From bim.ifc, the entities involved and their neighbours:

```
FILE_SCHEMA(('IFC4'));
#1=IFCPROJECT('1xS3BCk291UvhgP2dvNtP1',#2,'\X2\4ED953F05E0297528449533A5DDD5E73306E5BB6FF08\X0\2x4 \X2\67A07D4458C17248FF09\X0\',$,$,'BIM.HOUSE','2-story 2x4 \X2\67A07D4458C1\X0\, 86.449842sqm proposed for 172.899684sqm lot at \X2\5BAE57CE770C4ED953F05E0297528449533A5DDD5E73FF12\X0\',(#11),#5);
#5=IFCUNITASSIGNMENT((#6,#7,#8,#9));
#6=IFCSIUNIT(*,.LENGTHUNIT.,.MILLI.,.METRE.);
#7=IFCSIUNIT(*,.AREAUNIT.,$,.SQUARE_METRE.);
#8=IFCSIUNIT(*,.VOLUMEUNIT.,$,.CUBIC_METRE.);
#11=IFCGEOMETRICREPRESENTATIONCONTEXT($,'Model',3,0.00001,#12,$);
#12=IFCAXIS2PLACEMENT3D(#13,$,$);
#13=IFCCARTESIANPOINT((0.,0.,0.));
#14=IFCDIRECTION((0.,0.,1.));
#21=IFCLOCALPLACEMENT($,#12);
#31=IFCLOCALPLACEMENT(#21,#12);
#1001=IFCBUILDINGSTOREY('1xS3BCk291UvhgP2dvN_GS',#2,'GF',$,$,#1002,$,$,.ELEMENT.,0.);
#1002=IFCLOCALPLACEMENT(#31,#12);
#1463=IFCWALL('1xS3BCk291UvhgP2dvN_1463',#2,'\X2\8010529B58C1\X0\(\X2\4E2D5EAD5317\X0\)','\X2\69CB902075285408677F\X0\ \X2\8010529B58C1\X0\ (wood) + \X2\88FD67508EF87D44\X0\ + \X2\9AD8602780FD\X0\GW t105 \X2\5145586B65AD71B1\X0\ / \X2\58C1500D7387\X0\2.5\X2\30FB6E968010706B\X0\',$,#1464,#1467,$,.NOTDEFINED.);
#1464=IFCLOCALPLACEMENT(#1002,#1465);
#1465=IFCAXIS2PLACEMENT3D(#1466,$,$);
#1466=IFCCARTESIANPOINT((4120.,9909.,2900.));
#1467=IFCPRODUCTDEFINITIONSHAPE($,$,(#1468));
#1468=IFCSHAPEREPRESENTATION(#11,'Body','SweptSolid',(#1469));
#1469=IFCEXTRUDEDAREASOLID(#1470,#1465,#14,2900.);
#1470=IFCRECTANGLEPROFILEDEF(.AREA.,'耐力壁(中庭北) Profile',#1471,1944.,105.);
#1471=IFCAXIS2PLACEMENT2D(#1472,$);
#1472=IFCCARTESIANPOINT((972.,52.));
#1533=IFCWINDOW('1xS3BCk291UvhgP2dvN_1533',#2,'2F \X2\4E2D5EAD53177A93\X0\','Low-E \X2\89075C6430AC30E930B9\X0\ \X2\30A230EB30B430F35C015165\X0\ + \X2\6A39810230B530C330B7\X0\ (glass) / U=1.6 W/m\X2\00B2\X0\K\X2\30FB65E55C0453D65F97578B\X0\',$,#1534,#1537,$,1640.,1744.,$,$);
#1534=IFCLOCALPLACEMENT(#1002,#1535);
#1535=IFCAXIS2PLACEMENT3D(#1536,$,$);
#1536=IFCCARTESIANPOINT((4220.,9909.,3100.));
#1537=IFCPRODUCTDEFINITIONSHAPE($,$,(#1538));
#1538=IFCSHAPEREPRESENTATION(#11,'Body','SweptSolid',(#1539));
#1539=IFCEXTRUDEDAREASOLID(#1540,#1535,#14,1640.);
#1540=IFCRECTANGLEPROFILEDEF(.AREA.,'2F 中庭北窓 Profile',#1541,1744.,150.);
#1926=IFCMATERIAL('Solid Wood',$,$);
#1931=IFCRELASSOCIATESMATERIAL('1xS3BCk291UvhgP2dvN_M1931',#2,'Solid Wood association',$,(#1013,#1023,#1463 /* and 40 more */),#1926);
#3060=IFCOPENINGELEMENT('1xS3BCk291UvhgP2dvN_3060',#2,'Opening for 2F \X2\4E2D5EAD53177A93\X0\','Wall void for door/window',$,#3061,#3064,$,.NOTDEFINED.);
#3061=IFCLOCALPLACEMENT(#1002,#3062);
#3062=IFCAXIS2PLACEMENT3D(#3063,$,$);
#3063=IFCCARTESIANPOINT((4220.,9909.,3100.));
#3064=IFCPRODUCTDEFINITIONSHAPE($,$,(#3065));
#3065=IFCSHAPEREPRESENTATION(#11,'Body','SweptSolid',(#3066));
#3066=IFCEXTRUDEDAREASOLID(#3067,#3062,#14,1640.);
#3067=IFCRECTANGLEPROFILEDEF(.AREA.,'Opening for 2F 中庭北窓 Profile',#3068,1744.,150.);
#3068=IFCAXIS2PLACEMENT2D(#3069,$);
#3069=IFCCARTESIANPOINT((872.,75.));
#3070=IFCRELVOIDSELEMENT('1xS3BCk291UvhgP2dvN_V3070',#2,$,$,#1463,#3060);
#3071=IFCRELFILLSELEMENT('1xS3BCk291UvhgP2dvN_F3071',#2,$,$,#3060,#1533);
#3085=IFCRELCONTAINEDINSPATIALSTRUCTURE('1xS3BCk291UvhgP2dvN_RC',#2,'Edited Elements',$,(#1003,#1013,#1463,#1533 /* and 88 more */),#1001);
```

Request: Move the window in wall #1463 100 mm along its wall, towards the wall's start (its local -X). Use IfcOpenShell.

```python
import ifcopenshell
import ifcopenshell.api.geometry
import ifcopenshell.util.placement

model = ifcopenshell.open("bim.ifc")

window = model.by_guid("1xS3BCk291UvhgP2dvN_1533")
opening = window.FillsVoids[0].RelatingOpeningElement
wall = opening.VoidsElements[0].RelatingBuildingElement

wall_matrix = ifcopenshell.util.placement.get_local_placement(wall.ObjectPlacement)
shift = wall_matrix[:3, 0] * -100.0
before = ifcopenshell.util.placement.get_local_placement(window.ObjectPlacement)[:3, 3].copy()

# The window is not placed relative to its opening, so move both.
for product in (opening, window):
    matrix = ifcopenshell.util.placement.get_local_placement(product.ObjectPlacement)
    matrix[:3, 3] += shift
    ifcopenshell.api.geometry.edit_object_placement(model, product=product, matrix=matrix, is_si=False)

after = ifcopenshell.util.placement.get_local_placement(window.ObjectPlacement)[:3, 3]
print("window moved by", (after - before).round(3) + 0.0)

model.write("bim-out.ifc")
```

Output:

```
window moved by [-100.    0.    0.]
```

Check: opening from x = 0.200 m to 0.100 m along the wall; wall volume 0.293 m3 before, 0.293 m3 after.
